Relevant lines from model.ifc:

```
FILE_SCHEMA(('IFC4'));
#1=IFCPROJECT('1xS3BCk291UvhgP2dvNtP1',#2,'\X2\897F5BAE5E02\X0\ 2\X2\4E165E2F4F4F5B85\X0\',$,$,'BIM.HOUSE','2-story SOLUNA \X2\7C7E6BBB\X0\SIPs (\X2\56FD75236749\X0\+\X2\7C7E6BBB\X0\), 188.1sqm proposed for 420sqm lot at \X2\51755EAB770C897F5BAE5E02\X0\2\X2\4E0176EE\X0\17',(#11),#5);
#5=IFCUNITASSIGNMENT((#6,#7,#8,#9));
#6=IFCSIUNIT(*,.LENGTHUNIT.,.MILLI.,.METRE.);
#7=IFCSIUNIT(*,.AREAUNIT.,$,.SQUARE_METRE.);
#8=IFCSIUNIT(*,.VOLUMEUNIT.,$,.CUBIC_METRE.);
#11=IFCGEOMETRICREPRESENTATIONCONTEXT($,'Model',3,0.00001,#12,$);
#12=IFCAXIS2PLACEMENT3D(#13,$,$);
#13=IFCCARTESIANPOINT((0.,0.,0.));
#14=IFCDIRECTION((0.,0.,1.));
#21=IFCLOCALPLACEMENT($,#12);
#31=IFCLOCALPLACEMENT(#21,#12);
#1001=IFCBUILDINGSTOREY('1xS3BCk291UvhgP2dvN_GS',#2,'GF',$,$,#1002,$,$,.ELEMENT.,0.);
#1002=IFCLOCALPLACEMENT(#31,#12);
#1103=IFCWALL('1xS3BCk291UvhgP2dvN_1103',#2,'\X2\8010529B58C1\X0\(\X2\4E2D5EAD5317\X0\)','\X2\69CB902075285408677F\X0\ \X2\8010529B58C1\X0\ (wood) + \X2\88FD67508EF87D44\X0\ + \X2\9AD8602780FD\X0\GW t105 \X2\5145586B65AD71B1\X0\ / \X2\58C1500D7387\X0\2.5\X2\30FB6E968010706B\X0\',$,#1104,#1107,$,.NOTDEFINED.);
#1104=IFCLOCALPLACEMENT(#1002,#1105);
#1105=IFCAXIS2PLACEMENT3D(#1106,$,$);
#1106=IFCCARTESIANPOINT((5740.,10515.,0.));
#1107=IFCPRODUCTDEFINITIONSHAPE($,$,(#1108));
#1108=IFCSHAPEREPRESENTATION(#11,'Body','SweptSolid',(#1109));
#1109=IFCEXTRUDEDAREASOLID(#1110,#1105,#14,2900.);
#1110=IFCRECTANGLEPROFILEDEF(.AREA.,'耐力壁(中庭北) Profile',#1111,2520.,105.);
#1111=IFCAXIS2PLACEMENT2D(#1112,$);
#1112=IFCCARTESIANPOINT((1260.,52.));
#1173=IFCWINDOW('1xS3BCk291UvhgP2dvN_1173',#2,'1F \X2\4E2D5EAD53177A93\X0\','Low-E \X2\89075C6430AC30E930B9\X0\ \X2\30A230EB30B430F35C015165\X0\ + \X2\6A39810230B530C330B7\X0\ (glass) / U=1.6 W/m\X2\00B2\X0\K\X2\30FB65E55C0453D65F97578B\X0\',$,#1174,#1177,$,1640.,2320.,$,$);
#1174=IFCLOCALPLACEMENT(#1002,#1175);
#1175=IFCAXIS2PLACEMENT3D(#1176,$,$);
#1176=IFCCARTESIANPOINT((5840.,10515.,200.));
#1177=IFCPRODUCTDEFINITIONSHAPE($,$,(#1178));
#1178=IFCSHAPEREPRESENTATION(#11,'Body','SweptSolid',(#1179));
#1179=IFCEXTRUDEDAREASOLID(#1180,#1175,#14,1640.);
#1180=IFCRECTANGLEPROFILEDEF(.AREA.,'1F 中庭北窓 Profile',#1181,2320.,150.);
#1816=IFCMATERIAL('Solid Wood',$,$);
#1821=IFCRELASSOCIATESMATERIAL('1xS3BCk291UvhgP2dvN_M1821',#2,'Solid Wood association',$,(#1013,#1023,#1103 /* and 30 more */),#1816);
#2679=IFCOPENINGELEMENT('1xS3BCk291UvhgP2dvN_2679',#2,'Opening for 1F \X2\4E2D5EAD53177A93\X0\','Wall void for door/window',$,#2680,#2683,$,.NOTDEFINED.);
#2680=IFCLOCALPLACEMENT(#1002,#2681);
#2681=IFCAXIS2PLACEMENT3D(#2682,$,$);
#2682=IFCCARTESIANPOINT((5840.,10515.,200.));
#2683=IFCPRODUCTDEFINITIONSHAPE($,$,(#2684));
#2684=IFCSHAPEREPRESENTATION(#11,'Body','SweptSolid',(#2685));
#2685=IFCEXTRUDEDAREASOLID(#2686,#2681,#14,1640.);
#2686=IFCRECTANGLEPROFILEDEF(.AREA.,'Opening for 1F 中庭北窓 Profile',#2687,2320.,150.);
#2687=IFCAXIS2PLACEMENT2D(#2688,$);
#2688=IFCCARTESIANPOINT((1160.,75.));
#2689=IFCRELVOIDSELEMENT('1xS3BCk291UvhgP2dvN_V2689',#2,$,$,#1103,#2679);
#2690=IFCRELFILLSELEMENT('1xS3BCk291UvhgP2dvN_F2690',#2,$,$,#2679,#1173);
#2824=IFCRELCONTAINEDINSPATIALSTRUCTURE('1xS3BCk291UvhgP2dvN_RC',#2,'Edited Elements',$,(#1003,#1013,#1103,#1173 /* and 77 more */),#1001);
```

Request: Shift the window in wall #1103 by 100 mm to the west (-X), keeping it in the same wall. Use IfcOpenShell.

```python
import ifcopenshell
import ifcopenshell.api.geometry
import ifcopenshell.util.placement
import ifcopenshell.util.unit

model = ifcopenshell.open("model.ifc")
unit_scale = ifcopenshell.util.unit.calculate_unit_scale(model)

window = model.by_id(1173)
opening = window.FillsVoids[0].RelatingOpeningElement
wall = opening.VoidsElements[0].RelatingBuildingElement

wall_matrix = ifcopenshell.util.placement.get_local_placement(wall.ObjectPlacement)
shift = wall_matrix[:3, 0] * -0.1 / unit_scale
before = ifcopenshell.util.placement.get_local_placement(window.ObjectPlacement)[:3, 3].copy()

# The window is not placed relative to its opening, so move both.
for product in (opening, window):
    matrix = ifcopenshell.util.placement.get_local_placement(product.ObjectPlacement)
    matrix[:3, 3] += shift
    ifcopenshell.api.geometry.edit_object_placement(model, product=product, matrix=matrix, is_si=False)

after = ifcopenshell.util.placement.get_local_placement(window.ObjectPlacement)[:3, 3]
print("window moved by", (after - before).round(3) + 0.0)

model.write("model_rev.ifc")
```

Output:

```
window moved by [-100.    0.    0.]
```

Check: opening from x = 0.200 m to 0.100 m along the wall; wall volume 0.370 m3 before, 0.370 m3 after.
